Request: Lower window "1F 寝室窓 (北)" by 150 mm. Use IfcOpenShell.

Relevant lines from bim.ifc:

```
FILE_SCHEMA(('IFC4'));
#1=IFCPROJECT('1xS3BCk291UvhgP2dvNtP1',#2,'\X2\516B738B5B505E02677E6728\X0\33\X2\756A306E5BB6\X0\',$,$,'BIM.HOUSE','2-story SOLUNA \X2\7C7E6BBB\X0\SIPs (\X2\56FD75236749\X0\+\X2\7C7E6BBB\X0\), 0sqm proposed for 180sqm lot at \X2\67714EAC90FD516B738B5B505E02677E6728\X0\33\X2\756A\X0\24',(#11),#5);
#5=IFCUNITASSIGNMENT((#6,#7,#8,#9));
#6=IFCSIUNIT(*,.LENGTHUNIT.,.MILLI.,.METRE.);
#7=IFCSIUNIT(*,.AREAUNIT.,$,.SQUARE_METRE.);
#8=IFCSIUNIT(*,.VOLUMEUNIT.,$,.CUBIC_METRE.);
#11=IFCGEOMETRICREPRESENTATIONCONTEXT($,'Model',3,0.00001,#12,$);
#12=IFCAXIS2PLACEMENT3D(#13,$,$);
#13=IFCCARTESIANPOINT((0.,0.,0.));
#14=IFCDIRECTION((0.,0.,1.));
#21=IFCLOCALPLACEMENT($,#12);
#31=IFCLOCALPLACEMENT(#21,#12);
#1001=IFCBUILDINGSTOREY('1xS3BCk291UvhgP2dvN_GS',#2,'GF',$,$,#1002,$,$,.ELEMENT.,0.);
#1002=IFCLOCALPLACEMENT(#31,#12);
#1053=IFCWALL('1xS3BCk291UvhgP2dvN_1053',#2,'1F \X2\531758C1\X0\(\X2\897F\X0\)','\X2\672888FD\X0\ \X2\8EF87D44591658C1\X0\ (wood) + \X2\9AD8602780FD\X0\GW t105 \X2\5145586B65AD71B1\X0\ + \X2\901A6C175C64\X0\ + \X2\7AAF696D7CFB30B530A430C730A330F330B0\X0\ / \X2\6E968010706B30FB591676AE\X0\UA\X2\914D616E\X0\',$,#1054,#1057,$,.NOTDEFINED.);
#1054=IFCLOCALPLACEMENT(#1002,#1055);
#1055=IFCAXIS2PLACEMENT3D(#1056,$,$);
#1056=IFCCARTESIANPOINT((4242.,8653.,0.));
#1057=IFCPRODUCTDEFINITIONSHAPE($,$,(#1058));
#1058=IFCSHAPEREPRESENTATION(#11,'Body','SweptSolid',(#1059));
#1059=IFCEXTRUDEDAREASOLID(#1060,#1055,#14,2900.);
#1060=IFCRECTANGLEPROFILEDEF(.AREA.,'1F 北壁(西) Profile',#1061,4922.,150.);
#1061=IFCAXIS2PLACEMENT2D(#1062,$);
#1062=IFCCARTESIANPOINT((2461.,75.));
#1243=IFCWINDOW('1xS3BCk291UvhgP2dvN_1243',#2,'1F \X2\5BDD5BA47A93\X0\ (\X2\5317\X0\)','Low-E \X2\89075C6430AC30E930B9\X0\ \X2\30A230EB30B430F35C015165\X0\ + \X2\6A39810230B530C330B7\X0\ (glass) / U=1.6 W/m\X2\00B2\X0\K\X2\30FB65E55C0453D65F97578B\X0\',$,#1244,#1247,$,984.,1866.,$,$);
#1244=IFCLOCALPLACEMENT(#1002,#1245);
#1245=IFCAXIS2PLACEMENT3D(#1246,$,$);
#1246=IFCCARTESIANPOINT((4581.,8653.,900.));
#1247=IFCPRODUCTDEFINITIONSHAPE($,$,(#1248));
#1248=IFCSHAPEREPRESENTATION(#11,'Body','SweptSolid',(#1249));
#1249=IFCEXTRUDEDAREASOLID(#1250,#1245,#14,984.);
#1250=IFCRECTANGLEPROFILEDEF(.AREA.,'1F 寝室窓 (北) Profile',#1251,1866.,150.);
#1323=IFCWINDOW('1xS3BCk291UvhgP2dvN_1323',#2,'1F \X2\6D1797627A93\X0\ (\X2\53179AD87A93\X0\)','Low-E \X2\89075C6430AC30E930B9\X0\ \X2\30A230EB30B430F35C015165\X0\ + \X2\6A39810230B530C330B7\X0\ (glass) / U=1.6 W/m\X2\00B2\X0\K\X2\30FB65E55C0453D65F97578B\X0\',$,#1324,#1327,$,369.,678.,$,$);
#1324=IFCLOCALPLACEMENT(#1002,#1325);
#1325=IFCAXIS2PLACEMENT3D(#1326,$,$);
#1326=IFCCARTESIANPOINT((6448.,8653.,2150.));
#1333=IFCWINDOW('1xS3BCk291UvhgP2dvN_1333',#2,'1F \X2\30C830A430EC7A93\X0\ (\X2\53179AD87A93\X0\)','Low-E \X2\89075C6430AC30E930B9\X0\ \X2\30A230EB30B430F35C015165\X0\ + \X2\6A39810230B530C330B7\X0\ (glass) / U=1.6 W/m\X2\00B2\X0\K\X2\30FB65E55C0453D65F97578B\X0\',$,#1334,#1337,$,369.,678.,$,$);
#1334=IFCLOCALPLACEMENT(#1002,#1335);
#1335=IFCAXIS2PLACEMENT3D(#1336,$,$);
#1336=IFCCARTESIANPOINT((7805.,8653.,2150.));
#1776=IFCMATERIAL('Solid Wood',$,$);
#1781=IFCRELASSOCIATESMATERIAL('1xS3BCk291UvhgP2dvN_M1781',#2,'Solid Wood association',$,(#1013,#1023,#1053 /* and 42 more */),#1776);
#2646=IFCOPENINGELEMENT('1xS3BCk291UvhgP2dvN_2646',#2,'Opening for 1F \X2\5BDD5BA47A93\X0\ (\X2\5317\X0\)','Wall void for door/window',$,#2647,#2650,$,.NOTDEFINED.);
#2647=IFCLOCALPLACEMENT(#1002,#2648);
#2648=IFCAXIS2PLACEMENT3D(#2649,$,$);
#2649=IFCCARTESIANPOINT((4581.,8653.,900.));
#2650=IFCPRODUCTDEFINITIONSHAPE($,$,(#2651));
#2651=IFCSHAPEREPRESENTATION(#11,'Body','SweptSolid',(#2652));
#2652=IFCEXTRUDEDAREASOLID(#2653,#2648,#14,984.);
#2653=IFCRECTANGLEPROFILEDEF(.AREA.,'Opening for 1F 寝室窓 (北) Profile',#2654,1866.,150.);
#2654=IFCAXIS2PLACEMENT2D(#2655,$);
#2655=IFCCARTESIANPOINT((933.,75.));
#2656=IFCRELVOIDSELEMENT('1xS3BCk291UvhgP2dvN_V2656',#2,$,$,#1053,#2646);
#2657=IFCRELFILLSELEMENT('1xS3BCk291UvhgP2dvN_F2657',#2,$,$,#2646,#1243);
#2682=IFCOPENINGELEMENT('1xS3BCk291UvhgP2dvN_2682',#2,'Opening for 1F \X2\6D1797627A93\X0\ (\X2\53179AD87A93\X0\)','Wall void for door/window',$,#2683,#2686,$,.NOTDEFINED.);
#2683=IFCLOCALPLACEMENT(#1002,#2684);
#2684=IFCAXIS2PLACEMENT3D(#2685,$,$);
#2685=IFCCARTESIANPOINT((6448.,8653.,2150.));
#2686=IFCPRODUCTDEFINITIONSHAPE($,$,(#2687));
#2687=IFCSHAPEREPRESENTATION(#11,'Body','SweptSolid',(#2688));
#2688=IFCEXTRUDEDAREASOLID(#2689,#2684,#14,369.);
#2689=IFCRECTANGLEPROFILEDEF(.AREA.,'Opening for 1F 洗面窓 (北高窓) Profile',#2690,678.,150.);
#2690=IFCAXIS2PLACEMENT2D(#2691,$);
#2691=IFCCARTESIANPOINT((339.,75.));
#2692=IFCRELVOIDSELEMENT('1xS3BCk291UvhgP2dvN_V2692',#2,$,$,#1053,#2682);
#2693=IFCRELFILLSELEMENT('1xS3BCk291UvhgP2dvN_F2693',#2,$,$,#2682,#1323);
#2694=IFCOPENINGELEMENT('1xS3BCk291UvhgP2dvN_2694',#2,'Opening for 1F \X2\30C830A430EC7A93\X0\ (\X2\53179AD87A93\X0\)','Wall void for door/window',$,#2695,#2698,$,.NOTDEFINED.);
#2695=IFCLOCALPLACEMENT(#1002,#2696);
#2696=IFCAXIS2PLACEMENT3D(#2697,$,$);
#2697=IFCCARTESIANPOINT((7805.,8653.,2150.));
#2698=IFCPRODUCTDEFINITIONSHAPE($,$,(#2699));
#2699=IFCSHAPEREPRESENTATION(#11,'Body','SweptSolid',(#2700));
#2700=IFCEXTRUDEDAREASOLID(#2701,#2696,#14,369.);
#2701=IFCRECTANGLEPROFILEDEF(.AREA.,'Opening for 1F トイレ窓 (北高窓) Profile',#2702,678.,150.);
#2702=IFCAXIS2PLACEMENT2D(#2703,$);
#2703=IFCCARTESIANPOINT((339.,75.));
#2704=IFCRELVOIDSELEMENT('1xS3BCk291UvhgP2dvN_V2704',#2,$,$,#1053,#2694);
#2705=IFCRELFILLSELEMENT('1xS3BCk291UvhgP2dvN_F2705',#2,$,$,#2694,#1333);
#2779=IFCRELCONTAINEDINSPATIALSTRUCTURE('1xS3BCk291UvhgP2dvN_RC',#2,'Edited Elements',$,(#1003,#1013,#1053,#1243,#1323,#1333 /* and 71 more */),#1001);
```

```python
import numpy as np
import ifcopenshell
import ifcopenshell.api.geometry
import ifcopenshell.util.placement
import ifcopenshell.util.unit

model = ifcopenshell.open("bim.ifc")
unit_scale = ifcopenshell.util.unit.calculate_unit_scale(model)

window = model.by_guid("1xS3BCk291UvhgP2dvN_1243")
opening = window.FillsVoids[0].RelatingOpeningElement
dz = -150.0

shift = np.array([0.0, 0.0, dz])
# The window is not placed relative to its opening, so move both.
for product in (opening, window):
    matrix = ifcopenshell.util.placement.get_local_placement(product.ObjectPlacement)
    matrix[:3, 3] += shift
    ifcopenshell.api.geometry.edit_object_placement(model, product=product, matrix=matrix, is_si=False)

print(f"moved by {dz * unit_scale:+.3f} m")

model.write("bim_updated.ifc")
```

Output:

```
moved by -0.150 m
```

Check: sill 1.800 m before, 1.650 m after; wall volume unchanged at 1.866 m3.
